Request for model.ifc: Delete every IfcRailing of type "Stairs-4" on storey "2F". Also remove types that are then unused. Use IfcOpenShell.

First a look at what the model holds.

```python
import ifcopenshell
import ifcopenshell.util.element

model = ifcopenshell.open("model.ifc")
print(model.schema)
storey = next(s for s in model.by_type("IfcBuildingStorey") if s.Name == "2F")
railings = [e for e in ifcopenshell.util.element.get_decomposition(storey) if e.is_a("IfcRailing")]
seen = {}
for e in railings:
    element_type = ifcopenshell.util.element.get_type(e)
    name = element_type.Name if element_type not in (None, e) else None
    seen[name] = seen.get(name, 0) + 1
for name, count in sorted(seen.items(), key=str):
    print(count, "x", name)
```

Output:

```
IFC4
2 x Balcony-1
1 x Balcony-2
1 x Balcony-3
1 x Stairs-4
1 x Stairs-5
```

```python
import ifcopenshell
import ifcopenshell.api.root
import ifcopenshell.util.element

model = ifcopenshell.open("model.ifc")

storey = next(s for s in model.by_type("IfcBuildingStorey") if s.Name == "2F")
railings = [e for e in ifcopenshell.util.element.get_decomposition(storey) if e.is_a("IfcRailing")]
targets = [e for e in railings if (t := ifcopenshell.util.element.get_type(e)) not in (None, e) and t.Name == "Stairs-4"]
types = {ifcopenshell.util.element.get_type(e) for e in targets} - {None, *targets}

for e in targets:
    ifcopenshell.api.root.remove_product(model, product=e)
print(len(targets), "removed")

unused = [t for t in types if not ifcopenshell.util.element.get_types(t)]
for t in unused:
    ifcopenshell.api.root.remove_product(model, product=t)
print(len(unused), "unused types removed")

model.write("model_updated.ifc")
```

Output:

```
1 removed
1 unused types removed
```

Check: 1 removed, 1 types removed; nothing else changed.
